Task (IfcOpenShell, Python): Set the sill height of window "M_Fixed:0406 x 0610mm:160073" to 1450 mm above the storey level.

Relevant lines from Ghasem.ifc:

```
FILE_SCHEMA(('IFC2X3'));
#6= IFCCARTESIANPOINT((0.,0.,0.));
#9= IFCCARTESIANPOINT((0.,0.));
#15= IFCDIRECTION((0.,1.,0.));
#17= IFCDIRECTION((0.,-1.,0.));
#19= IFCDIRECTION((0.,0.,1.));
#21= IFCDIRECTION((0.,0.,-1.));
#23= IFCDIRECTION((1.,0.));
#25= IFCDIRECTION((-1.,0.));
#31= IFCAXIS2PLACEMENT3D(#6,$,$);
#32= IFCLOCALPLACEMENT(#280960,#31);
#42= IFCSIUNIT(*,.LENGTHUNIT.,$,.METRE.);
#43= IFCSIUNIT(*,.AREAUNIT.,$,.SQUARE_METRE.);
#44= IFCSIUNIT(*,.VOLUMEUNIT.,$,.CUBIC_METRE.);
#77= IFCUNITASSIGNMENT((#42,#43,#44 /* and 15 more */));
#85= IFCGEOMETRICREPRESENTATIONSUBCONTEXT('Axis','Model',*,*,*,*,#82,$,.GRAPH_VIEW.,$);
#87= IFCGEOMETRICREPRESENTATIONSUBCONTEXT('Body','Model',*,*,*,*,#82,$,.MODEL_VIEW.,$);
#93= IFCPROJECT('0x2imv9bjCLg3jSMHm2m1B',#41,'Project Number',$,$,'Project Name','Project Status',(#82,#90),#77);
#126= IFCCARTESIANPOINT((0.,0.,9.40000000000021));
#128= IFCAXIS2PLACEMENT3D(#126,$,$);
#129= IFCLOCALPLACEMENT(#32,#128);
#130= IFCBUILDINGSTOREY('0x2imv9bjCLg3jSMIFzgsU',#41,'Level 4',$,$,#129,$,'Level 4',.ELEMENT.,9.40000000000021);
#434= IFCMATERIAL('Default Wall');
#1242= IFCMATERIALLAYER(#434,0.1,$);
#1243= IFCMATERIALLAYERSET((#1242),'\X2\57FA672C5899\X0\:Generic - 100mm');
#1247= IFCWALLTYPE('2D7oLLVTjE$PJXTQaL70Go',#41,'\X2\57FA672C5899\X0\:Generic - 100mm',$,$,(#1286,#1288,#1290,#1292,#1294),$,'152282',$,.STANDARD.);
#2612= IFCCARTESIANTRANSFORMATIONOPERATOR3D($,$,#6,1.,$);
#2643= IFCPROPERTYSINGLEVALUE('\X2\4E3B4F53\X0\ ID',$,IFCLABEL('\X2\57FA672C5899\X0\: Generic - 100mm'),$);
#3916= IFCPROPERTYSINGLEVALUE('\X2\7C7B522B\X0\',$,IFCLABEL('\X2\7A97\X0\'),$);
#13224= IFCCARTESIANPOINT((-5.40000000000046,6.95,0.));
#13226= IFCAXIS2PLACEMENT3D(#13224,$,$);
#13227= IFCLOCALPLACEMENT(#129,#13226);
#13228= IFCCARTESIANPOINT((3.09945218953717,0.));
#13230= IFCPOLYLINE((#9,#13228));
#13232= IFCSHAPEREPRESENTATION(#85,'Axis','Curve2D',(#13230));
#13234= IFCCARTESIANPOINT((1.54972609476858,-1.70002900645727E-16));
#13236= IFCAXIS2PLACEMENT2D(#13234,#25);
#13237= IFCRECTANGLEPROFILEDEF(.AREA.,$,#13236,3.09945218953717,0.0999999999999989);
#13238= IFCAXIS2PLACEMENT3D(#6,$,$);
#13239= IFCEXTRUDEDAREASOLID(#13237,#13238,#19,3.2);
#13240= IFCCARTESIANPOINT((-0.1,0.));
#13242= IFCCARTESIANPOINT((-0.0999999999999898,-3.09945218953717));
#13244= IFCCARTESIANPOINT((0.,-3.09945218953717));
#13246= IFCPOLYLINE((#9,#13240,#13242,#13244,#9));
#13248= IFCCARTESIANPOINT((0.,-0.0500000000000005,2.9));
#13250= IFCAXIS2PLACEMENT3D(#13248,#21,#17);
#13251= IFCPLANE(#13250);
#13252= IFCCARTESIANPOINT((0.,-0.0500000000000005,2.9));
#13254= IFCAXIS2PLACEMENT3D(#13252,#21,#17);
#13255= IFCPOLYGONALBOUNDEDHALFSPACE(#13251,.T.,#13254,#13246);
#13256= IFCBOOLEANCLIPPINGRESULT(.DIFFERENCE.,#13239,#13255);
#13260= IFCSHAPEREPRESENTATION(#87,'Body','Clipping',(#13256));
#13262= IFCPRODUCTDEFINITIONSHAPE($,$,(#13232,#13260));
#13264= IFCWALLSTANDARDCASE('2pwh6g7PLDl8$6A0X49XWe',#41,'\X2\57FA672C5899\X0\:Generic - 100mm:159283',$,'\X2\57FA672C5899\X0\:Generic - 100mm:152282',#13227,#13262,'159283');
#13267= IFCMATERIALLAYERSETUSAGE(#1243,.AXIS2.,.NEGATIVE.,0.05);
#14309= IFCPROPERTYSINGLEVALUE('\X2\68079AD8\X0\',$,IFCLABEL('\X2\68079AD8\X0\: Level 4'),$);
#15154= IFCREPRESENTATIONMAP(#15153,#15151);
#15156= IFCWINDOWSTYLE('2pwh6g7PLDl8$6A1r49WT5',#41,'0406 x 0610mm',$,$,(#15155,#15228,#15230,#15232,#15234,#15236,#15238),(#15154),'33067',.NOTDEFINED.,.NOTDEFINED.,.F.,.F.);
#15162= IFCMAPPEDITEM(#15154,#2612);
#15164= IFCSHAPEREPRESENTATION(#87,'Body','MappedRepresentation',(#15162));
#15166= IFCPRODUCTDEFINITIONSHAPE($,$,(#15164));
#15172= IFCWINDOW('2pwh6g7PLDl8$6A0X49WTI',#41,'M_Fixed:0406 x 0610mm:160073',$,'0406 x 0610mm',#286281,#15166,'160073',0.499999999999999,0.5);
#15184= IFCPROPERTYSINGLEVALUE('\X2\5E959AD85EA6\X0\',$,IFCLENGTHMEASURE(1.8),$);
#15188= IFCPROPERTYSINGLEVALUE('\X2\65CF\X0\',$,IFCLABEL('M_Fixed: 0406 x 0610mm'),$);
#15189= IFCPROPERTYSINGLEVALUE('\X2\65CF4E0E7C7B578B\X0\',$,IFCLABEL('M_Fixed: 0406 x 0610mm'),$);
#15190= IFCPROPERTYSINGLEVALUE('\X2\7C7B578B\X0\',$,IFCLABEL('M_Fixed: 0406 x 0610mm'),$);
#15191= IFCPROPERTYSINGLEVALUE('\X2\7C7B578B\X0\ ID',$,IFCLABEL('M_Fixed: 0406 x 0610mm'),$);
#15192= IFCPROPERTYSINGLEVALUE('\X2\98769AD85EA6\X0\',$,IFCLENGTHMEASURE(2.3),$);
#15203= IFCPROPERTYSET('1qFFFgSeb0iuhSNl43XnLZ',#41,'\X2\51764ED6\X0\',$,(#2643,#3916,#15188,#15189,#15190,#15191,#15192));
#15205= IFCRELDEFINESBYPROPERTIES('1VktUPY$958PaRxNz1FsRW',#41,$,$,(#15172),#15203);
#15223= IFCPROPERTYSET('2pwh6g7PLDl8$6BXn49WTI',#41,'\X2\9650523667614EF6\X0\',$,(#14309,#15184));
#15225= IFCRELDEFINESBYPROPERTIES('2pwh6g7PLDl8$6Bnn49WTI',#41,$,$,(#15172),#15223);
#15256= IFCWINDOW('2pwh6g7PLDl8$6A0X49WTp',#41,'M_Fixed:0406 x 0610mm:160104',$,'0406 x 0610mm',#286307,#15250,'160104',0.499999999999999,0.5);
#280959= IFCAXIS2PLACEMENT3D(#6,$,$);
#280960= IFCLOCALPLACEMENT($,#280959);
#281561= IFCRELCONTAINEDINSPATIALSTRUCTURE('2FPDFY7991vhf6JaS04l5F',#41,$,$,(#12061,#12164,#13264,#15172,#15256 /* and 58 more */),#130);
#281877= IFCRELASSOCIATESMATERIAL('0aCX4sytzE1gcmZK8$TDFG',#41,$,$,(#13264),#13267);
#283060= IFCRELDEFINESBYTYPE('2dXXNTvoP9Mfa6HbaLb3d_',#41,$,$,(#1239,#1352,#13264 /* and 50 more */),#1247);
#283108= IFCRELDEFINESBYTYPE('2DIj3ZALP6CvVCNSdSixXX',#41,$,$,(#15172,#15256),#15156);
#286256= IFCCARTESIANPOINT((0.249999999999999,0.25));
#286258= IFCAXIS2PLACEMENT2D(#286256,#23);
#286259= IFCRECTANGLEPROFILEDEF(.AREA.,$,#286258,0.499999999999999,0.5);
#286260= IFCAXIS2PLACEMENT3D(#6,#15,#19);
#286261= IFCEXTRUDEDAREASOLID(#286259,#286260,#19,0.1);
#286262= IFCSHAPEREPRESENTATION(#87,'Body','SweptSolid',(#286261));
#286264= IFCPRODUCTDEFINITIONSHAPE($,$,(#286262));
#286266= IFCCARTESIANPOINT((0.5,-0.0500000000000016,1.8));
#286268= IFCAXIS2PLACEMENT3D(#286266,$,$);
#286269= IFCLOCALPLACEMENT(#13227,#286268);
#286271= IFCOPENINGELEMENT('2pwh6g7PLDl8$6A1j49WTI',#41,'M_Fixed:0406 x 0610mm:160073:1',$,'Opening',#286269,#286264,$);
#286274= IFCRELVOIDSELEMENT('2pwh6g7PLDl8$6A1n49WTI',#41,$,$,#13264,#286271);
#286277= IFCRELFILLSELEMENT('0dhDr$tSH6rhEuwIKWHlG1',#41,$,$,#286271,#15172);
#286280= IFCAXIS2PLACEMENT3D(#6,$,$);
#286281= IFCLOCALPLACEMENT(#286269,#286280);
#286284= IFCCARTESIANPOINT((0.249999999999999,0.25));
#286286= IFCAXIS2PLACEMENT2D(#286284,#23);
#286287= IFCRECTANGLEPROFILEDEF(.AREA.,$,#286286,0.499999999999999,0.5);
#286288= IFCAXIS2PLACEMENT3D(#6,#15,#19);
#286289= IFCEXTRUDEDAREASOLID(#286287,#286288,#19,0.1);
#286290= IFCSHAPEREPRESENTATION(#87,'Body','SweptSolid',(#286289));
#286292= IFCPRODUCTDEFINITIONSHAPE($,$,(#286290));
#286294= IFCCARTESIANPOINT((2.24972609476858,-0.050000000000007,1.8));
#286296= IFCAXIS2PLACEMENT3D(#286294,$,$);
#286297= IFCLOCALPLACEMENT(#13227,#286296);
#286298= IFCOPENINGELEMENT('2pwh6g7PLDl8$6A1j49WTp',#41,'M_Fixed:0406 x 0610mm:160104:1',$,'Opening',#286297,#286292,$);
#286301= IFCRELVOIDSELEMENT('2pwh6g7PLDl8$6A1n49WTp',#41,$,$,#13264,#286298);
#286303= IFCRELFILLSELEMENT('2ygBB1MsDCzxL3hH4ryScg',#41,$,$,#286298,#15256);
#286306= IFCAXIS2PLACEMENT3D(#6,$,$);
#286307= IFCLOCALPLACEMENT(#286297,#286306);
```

```python
import numpy as np
import ifcopenshell
import ifcopenshell.api.geometry
import ifcopenshell.api.pset
import ifcopenshell.geom
import ifcopenshell.util.element
import ifcopenshell.util.placement
import ifcopenshell.util.shape
import ifcopenshell.util.unit

model = ifcopenshell.open("Ghasem.ifc")
unit_scale = ifcopenshell.util.unit.calculate_unit_scale(model)

window = model.by_guid("2pwh6g7PLDl8$6A0X49WTI")
opening = window.FillsVoids[0].RelatingOpeningElement
storey = ifcopenshell.util.element.get_container(window, ifc_class="IfcBuildingStorey")
level = ifcopenshell.util.placement.get_local_placement(storey.ObjectPlacement)[2, 3]

# The opening's origin need not be at the sill, so measure its lowest point.
shape = ifcopenshell.geom.create_shape(ifcopenshell.geom.settings(), opening)
bottom = ifcopenshell.util.shape.get_shape_bottom_elevation(shape, shape.geometry) / unit_scale
dz = level + 1.45 / unit_scale - bottom

shift = np.array([0.0, 0.0, dz])
# The window is placed relative to its opening, so it follows when the opening moves.
matrix = ifcopenshell.util.placement.get_local_placement(opening.ObjectPlacement)
matrix[:3, 3] += shift
ifcopenshell.api.geometry.edit_object_placement(
    model, product=opening, matrix=matrix, is_si=False, should_transform_children=True
)

# Keep the stored heights in step.
pset = model.by_id(ifcopenshell.util.element.get_pset(window, "其他", should_inherit=False)["id"])
ifcopenshell.api.pset.edit_pset(model, pset=pset, properties={
    "顶高度": model.create_entity("IfcLengthMeasure", ifcopenshell.util.element.get_pset(window, "其他", "顶高度") + dz),
})
pset = model.by_id(ifcopenshell.util.element.get_pset(window, "限制条件", should_inherit=False)["id"])
ifcopenshell.api.pset.edit_pset(model, pset=pset, properties={
    "底高度": model.create_entity("IfcLengthMeasure", ifcopenshell.util.element.get_pset(window, "限制条件", "底高度") + dz),
})

print(f"moved by {dz * unit_scale:+.3f} m")

model.write("Ghasem_v2.ifc")
```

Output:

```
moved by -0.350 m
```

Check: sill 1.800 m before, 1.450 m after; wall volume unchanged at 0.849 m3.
